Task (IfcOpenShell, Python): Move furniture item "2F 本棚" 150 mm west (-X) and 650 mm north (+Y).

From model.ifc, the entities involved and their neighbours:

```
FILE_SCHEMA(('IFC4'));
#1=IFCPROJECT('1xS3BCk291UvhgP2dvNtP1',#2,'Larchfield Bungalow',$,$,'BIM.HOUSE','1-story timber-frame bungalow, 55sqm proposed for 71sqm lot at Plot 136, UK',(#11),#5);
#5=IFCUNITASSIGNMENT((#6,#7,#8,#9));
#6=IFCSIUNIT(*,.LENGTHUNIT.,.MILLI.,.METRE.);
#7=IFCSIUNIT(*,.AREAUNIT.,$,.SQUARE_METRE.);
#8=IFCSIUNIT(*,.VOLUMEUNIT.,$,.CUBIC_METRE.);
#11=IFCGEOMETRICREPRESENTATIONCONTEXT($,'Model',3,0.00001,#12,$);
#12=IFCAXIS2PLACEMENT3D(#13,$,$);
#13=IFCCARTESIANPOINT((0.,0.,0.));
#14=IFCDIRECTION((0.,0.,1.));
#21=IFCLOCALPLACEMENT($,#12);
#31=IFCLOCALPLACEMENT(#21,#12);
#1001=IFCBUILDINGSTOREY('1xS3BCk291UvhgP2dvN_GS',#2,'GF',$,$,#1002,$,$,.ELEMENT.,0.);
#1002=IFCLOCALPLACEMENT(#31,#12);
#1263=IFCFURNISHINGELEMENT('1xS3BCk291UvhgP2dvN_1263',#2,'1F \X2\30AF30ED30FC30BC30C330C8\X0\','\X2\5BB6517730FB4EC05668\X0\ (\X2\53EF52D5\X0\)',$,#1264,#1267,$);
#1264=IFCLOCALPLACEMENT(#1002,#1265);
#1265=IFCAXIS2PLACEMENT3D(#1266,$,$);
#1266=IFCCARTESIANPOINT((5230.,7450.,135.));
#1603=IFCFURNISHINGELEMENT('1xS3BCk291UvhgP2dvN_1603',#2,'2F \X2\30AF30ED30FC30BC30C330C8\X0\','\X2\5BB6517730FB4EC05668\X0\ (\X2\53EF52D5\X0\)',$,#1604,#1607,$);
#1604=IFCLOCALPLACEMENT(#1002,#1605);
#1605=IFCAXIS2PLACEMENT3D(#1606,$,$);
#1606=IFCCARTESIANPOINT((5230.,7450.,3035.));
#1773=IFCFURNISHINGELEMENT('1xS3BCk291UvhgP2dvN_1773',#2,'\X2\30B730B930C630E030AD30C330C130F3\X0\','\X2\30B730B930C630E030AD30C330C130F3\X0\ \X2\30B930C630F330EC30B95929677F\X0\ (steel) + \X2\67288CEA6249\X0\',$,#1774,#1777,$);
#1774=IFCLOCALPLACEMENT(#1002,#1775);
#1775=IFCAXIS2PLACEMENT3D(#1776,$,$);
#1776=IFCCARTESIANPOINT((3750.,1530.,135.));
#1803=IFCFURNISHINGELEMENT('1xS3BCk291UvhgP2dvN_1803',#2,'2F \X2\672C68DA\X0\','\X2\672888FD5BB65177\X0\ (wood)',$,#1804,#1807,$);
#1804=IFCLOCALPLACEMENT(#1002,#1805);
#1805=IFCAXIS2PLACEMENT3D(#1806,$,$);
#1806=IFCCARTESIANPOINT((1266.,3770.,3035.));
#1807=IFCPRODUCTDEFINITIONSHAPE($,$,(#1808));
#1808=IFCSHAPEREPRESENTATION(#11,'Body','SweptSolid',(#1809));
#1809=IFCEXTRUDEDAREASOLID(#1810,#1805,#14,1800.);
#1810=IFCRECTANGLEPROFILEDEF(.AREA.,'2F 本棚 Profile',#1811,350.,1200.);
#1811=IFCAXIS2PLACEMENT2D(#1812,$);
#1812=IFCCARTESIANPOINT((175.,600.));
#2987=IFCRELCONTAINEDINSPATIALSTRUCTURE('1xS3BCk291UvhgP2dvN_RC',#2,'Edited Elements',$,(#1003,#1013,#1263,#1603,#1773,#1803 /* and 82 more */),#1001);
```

```python
import ifcopenshell
import ifcopenshell.api.geometry
import ifcopenshell.util.placement

model = ifcopenshell.open("model.ifc")

item = model.by_guid("1xS3BCk291UvhgP2dvN_1803")
matrix = ifcopenshell.util.placement.get_local_placement(item.ObjectPlacement)
matrix[0, 3] -= 150.0
matrix[1, 3] += 650.0
ifcopenshell.api.geometry.edit_object_placement(model, product=item, matrix=matrix, is_si=False)

print(ifcopenshell.util.placement.get_local_placement(item.ObjectPlacement).round(3) + 0.0)

model.write("model_v2.ifc")
```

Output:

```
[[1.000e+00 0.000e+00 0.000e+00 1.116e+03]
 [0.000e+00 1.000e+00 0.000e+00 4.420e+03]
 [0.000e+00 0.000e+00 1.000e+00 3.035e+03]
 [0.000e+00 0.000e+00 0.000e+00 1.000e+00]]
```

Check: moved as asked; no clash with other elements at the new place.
